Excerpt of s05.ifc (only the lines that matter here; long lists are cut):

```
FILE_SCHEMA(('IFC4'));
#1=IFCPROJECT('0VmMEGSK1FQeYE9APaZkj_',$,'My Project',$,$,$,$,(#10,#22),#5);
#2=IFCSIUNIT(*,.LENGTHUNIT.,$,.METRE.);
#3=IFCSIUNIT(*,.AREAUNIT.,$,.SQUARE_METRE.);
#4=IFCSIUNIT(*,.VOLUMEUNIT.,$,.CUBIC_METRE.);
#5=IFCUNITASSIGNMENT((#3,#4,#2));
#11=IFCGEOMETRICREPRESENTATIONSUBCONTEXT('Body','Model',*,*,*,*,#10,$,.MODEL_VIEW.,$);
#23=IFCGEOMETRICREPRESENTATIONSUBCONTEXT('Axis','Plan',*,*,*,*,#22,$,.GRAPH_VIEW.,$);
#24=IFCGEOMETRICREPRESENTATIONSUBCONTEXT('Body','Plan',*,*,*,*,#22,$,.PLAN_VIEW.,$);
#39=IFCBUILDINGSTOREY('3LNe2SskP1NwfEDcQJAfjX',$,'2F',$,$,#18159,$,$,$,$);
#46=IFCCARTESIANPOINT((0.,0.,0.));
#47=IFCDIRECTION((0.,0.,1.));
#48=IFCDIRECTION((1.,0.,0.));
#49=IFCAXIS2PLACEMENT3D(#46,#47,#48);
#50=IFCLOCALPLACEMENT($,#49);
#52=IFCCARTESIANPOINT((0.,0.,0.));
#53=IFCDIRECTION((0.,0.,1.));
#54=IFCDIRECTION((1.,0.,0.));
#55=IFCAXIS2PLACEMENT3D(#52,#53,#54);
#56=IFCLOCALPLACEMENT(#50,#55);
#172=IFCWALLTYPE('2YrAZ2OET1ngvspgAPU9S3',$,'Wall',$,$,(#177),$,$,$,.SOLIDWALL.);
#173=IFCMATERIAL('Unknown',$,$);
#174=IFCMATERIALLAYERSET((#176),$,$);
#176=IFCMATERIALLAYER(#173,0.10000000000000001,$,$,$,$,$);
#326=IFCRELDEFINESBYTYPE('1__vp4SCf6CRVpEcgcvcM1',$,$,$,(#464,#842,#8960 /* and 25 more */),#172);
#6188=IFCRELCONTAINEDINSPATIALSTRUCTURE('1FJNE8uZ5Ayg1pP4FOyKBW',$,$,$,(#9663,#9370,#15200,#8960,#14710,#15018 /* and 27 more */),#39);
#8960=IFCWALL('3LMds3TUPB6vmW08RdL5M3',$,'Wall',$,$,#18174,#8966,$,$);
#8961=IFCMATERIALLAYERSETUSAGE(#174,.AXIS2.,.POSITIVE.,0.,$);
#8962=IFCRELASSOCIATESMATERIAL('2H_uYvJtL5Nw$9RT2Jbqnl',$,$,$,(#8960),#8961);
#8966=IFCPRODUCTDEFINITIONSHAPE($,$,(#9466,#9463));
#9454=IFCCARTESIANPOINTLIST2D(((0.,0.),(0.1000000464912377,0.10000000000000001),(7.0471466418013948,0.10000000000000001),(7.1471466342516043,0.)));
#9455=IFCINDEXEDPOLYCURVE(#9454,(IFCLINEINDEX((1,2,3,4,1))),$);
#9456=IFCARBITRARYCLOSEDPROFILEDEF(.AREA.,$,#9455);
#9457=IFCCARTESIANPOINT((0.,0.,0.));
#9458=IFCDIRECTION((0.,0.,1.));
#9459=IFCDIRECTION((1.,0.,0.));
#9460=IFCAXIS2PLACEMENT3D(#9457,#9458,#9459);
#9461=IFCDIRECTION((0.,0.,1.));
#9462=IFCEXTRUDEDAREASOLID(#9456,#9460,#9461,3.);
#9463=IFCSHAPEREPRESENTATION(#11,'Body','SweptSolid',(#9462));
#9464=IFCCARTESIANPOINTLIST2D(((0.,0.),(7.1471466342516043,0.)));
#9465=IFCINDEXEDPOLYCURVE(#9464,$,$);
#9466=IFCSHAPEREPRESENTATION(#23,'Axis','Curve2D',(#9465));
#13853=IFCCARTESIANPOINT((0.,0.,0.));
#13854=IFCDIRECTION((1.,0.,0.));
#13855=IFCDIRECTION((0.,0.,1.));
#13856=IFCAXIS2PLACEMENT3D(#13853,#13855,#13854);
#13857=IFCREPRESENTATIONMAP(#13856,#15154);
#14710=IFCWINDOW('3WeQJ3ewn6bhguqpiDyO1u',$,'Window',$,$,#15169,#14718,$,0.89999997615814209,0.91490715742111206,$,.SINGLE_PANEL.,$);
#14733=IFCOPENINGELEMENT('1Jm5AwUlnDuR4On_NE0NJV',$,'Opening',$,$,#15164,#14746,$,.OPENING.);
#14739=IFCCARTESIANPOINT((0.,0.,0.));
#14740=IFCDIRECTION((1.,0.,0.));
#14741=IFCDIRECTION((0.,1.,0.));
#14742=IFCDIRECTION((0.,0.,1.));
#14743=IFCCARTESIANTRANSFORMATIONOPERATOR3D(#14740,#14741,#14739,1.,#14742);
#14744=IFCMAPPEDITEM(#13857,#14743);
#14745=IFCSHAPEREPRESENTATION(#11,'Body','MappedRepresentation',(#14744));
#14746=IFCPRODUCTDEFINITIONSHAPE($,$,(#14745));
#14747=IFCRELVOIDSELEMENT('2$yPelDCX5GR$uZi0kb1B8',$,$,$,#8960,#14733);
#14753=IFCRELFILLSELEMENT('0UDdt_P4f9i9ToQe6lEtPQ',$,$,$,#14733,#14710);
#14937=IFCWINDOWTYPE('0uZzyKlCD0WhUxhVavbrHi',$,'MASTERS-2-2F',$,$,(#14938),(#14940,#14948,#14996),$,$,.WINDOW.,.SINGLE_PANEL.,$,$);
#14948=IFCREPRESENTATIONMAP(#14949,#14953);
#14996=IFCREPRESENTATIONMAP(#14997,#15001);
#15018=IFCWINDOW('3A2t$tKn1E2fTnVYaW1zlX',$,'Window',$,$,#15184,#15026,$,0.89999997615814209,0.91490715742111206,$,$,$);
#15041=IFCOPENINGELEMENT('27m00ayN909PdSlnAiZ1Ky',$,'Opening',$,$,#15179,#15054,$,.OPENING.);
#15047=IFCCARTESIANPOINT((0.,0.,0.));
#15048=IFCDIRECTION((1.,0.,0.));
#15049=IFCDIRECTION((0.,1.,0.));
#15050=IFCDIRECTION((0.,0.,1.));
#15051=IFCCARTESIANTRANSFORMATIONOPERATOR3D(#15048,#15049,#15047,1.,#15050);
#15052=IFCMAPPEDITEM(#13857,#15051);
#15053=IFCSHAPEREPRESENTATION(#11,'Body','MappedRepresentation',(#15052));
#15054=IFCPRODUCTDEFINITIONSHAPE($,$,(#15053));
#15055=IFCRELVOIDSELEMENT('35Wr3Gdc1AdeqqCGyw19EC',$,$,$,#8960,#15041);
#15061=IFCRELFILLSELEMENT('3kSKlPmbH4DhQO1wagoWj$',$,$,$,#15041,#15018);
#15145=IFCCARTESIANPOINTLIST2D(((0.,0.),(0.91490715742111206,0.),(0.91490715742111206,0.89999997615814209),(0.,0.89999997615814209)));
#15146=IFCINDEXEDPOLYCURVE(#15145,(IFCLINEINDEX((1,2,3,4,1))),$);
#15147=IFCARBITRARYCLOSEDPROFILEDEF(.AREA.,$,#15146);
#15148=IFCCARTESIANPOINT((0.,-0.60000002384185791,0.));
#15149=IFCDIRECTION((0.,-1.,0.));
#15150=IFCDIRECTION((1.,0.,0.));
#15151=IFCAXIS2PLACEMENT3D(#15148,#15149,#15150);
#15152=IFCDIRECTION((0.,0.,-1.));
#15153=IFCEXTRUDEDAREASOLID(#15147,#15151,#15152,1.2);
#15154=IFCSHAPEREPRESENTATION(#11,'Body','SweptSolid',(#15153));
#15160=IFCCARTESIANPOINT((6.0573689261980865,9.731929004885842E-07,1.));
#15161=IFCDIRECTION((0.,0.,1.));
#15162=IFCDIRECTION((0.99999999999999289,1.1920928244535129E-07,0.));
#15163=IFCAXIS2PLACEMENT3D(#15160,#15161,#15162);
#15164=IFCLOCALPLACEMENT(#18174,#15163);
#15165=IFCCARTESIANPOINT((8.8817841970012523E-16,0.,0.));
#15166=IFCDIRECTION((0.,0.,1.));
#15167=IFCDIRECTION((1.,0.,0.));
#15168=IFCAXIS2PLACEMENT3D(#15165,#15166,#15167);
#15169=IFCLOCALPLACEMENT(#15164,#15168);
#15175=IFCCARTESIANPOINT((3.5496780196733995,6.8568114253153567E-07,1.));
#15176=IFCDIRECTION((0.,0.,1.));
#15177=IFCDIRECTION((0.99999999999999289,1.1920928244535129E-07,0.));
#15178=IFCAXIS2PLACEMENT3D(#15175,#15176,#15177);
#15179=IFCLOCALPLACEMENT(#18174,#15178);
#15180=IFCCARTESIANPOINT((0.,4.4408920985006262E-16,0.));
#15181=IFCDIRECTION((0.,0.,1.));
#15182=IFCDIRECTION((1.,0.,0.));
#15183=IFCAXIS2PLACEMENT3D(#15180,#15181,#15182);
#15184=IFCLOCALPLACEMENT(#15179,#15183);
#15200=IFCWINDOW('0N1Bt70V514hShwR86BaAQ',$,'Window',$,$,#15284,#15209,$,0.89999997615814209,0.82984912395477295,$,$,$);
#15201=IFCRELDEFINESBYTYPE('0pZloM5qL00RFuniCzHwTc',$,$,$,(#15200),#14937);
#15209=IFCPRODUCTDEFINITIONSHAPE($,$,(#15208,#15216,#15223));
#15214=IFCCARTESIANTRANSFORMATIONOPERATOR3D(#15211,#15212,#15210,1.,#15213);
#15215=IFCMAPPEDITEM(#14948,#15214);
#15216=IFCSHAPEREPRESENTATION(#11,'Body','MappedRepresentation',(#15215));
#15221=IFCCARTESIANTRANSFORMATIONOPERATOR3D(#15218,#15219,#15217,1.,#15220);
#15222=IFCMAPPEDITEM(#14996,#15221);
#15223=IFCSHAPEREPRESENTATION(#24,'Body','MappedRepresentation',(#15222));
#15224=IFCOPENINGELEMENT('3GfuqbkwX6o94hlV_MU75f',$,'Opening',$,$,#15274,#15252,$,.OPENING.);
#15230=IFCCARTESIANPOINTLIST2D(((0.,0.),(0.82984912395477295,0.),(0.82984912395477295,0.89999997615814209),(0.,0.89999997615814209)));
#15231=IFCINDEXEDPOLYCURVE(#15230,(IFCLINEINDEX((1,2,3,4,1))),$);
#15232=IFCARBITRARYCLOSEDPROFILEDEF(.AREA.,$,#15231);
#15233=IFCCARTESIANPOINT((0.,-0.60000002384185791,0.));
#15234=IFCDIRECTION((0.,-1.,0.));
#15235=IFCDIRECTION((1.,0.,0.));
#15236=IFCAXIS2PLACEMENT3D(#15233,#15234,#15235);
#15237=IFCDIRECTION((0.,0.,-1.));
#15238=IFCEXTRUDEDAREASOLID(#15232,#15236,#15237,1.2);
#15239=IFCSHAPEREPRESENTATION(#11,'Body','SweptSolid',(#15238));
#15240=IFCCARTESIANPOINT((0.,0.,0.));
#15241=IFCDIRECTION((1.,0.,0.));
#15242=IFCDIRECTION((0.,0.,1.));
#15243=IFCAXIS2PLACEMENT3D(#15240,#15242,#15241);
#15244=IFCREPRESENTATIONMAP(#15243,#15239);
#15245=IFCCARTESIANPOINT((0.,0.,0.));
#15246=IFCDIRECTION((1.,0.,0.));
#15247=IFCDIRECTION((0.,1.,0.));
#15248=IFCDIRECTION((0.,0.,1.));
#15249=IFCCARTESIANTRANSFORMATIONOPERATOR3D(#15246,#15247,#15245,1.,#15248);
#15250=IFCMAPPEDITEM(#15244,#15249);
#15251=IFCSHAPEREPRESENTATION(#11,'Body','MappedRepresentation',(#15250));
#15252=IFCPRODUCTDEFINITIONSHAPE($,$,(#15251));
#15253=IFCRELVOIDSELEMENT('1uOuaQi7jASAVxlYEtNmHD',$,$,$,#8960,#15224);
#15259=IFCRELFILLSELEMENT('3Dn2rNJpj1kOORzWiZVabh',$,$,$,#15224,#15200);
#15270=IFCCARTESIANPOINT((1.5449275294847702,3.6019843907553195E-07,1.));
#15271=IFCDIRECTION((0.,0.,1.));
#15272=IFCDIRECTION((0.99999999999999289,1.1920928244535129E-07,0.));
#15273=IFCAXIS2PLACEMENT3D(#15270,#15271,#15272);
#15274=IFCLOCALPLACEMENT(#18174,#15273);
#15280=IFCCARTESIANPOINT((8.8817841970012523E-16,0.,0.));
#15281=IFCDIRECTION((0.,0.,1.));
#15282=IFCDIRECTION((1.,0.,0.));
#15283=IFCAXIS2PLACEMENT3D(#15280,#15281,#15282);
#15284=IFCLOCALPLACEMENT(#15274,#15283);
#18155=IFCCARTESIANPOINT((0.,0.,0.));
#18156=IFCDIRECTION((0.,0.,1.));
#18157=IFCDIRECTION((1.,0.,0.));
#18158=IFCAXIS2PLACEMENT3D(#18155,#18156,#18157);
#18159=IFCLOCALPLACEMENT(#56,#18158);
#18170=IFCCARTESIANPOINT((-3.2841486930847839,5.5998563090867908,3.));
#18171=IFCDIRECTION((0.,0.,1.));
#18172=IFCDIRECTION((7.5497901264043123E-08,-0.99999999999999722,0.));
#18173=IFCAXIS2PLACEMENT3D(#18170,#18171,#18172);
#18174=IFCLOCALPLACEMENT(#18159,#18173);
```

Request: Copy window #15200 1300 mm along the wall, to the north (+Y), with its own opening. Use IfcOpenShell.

```python
import ifcopenshell
import ifcopenshell.api.feature
import ifcopenshell.api.geometry
import ifcopenshell.api.root
import ifcopenshell.geom
import ifcopenshell.util.element
import ifcopenshell.util.placement
import ifcopenshell.util.shape

model = ifcopenshell.open("s05.ifc")
settings = ifcopenshell.geom.settings()


def volume(element):
    """Net volume in cubic metres, openings subtracted."""
    shape = ifcopenshell.geom.create_shape(settings, element)
    return ifcopenshell.util.shape.get_volume(shape.geometry)


window = model.by_guid("0N1Bt70V514hShwR86BaAQ")
opening = window.FillsVoids[0].RelatingOpeningElement
wall = opening.VoidsElements[0].RelatingBuildingElement
before = volume(wall)
shift = ifcopenshell.util.placement.get_local_placement(wall.ObjectPlacement)[:3, 0] * -1.3

# copy_class copies the void relationship, type, container and properties, but no geometry.
new_opening = ifcopenshell.api.root.copy_class(model, product=opening)
new_opening.Representation = ifcopenshell.util.element.copy_deep(
    model, opening.Representation, exclude=["IfcGeometricRepresentationContext", "IfcRepresentationMap"]
)
new_window = ifcopenshell.api.root.copy_class(model, product=window)
new_window.Representation = ifcopenshell.util.element.copy_deep(
    model, window.Representation, exclude=["IfcGeometricRepresentationContext", "IfcRepresentationMap"]
)
ifcopenshell.api.feature.add_filling(model, opening=new_opening, element=new_window)

for old, new in ((opening, new_opening), (window, new_window)):
    matrix = ifcopenshell.util.placement.get_local_placement(old.ObjectPlacement)
    matrix[:3, 3] += shift
    ifcopenshell.api.geometry.edit_object_placement(model, product=new, matrix=matrix, is_si=False)

after = volume(wall)

print(f"wall volume {before:.3f} -> {after:.3f} m3")

model.write("s05-out.ifc")
```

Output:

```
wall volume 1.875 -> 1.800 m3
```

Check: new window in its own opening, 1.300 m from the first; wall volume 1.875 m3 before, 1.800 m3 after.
